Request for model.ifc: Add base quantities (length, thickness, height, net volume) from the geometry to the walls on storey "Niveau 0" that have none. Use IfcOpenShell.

First a look at what the model holds.

```python
import ifcopenshell
import ifcopenshell.util.element
import ifcopenshell.util.unit

model = ifcopenshell.open("model.ifc")
print(model.schema)
for unit_type in ("LENGTHUNIT", "AREAUNIT", "VOLUMEUNIT"):
    print(unit_type, ifcopenshell.util.unit.calculate_unit_scale(model, unit_type))
storey = next(s for s in model.by_type("IfcBuildingStorey") if s.Name == "Niveau 0")
walls = [e for e in ifcopenshell.util.element.get_decomposition(storey) if e.is_a("IfcWall")]
for e in sorted(walls, key=lambda e: e.id()):
    print(e.id(), e.is_a(), e.Name, list(ifcopenshell.util.element.get_psets(e, qtos_only=True)), sep=" | ")
```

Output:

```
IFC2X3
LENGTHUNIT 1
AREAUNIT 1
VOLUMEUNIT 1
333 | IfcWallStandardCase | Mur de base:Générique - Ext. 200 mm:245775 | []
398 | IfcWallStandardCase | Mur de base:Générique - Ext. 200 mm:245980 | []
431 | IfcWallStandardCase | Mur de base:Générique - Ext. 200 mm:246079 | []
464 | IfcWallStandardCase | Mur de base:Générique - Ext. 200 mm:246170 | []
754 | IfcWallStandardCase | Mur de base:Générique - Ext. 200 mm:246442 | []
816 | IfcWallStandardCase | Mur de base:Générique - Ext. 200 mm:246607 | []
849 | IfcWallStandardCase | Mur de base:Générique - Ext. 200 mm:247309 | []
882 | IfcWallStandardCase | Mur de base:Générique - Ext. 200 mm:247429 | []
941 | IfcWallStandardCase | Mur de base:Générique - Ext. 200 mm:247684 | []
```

```python
import ifcopenshell
import ifcopenshell.api.pset
import ifcopenshell.geom
import ifcopenshell.util.element
import ifcopenshell.util.shape
import ifcopenshell.util.unit

model = ifcopenshell.open("model.ifc")
unit_scale = ifcopenshell.util.unit.calculate_unit_scale(model)
volume_scale = ifcopenshell.util.unit.calculate_unit_scale(model, "VOLUMEUNIT")
settings = ifcopenshell.geom.settings()

storey = next(s for s in model.by_type("IfcBuildingStorey") if s.Name == "Niveau 0")
walls = [e for e in ifcopenshell.util.element.get_decomposition(storey) if e.is_a("IfcWall")]

for e in sorted(walls, key=lambda e: e.id()):
    if ifcopenshell.util.element.get_psets(e, qtos_only=True, should_inherit=False):
        continue
    # Geometry comes back in metres, in the element's own axes.
    shape = ifcopenshell.geom.create_shape(settings, e)
    values = {
        "Length": ifcopenshell.util.shape.get_x(shape.geometry) / unit_scale,
        "Width": ifcopenshell.util.shape.get_y(shape.geometry) / unit_scale,
        "Height": ifcopenshell.util.shape.get_z(shape.geometry) / unit_scale,
        "NetVolume": ifcopenshell.util.shape.get_volume(shape.geometry) / volume_scale,
    }
    qto = ifcopenshell.api.pset.add_qto(model, product=e, name="BaseQuantities")
    ifcopenshell.api.pset.edit_qto(model, qto=qto, properties=values)
    print(e.id(), {k: round(v, 3) for k, v in values.items()})

model.write("model_edited.ifc")
```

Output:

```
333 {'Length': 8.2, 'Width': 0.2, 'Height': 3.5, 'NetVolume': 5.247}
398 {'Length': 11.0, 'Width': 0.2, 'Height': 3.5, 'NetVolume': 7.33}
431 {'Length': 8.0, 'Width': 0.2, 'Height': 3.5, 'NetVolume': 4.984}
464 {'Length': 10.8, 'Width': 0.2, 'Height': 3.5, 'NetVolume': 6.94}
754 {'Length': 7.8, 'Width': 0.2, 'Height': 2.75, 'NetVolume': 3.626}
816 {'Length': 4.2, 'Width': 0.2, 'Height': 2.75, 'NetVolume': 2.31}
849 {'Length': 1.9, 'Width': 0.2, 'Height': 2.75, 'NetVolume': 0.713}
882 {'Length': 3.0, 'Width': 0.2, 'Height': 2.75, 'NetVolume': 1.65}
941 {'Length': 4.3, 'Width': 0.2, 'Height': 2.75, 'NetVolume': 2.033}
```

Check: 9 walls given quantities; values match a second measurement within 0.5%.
